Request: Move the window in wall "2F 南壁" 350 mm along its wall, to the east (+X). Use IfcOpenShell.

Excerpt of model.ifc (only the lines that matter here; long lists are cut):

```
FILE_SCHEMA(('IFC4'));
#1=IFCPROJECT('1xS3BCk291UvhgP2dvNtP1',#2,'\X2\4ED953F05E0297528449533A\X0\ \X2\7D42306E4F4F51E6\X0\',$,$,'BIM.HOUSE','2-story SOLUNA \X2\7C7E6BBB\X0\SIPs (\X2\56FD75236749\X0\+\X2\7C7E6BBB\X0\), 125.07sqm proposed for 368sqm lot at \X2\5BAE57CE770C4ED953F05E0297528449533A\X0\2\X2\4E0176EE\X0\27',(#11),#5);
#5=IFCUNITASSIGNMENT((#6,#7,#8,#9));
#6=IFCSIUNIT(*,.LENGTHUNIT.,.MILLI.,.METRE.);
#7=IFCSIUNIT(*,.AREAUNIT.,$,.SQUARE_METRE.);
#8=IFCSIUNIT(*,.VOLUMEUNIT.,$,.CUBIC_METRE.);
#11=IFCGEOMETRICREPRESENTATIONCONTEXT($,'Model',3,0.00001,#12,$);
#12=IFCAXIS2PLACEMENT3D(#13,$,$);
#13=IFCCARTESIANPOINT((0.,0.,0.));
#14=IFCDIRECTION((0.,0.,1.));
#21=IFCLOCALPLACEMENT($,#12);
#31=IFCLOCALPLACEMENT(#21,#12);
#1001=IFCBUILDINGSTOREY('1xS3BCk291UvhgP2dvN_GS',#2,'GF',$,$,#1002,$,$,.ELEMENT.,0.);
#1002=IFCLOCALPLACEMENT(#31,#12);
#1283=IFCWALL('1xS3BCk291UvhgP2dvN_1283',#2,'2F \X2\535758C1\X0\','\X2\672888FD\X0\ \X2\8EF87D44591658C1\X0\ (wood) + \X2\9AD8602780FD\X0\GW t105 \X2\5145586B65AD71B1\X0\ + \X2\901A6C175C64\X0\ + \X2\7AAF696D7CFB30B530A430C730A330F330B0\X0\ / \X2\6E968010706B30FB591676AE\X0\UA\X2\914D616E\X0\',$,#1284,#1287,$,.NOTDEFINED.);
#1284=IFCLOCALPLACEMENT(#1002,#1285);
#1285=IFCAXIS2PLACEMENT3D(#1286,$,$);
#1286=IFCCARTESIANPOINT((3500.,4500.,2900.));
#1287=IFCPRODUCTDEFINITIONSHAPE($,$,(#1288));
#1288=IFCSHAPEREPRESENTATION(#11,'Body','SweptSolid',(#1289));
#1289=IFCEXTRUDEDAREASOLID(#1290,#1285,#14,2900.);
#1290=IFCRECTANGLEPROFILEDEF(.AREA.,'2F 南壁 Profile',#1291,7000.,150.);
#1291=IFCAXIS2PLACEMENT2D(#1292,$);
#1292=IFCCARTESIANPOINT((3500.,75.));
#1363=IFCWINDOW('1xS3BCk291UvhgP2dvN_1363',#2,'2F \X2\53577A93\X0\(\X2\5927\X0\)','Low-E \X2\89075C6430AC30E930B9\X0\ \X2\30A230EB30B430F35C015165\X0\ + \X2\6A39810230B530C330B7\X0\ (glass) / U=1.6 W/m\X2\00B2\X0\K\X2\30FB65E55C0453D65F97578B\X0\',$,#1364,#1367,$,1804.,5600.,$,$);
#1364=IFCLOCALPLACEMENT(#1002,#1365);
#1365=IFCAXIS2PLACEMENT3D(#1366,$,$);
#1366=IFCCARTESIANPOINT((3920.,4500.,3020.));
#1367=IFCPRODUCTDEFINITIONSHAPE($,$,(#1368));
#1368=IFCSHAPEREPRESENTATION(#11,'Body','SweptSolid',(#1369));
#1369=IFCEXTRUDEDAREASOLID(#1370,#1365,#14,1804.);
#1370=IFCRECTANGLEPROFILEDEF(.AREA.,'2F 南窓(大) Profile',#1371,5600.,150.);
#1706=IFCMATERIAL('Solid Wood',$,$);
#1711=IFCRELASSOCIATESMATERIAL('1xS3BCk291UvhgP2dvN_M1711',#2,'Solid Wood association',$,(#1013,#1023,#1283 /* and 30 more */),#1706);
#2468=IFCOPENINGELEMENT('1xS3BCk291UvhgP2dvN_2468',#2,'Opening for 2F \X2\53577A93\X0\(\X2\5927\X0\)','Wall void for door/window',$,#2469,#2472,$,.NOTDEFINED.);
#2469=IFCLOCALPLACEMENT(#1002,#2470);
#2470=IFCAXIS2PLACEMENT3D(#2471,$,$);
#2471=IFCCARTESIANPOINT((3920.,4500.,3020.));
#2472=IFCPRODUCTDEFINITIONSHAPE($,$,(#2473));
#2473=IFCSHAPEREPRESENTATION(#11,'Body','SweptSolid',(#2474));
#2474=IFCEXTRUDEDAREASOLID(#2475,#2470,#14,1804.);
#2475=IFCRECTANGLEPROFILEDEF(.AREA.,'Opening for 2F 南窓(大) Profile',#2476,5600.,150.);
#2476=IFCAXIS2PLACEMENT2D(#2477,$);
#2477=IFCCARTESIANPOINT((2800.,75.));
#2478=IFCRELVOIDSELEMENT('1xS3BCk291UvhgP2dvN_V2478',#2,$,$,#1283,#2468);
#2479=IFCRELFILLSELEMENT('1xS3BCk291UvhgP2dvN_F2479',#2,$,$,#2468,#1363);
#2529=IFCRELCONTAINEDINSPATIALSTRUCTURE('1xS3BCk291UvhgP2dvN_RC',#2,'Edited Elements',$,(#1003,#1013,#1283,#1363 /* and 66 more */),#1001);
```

```python
import ifcopenshell
import ifcopenshell.api.geometry
import ifcopenshell.util.placement
import ifcopenshell.util.unit

model = ifcopenshell.open("model.ifc")
unit_scale = ifcopenshell.util.unit.calculate_unit_scale(model)

window = model.by_guid("1xS3BCk291UvhgP2dvN_1363")
opening = window.FillsVoids[0].RelatingOpeningElement
wall = opening.VoidsElements[0].RelatingBuildingElement

wall_matrix = ifcopenshell.util.placement.get_local_placement(wall.ObjectPlacement)
shift = wall_matrix[:3, 0] * 0.35 / unit_scale
before = ifcopenshell.util.placement.get_local_placement(window.ObjectPlacement)[:3, 3].copy()

# The window is not placed relative to its opening, so move both.
for product in (opening, window):
    matrix = ifcopenshell.util.placement.get_local_placement(product.ObjectPlacement)
    matrix[:3, 3] += shift
    ifcopenshell.api.geometry.edit_object_placement(model, product=product, matrix=matrix, is_si=False)

after = ifcopenshell.util.placement.get_local_placement(window.ObjectPlacement)[:3, 3]
print("window moved by", (after - before).round(3) + 0.0)

model.write("model-out.ifc")
```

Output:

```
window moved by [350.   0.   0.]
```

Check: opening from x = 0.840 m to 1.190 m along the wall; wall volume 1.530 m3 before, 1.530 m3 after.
